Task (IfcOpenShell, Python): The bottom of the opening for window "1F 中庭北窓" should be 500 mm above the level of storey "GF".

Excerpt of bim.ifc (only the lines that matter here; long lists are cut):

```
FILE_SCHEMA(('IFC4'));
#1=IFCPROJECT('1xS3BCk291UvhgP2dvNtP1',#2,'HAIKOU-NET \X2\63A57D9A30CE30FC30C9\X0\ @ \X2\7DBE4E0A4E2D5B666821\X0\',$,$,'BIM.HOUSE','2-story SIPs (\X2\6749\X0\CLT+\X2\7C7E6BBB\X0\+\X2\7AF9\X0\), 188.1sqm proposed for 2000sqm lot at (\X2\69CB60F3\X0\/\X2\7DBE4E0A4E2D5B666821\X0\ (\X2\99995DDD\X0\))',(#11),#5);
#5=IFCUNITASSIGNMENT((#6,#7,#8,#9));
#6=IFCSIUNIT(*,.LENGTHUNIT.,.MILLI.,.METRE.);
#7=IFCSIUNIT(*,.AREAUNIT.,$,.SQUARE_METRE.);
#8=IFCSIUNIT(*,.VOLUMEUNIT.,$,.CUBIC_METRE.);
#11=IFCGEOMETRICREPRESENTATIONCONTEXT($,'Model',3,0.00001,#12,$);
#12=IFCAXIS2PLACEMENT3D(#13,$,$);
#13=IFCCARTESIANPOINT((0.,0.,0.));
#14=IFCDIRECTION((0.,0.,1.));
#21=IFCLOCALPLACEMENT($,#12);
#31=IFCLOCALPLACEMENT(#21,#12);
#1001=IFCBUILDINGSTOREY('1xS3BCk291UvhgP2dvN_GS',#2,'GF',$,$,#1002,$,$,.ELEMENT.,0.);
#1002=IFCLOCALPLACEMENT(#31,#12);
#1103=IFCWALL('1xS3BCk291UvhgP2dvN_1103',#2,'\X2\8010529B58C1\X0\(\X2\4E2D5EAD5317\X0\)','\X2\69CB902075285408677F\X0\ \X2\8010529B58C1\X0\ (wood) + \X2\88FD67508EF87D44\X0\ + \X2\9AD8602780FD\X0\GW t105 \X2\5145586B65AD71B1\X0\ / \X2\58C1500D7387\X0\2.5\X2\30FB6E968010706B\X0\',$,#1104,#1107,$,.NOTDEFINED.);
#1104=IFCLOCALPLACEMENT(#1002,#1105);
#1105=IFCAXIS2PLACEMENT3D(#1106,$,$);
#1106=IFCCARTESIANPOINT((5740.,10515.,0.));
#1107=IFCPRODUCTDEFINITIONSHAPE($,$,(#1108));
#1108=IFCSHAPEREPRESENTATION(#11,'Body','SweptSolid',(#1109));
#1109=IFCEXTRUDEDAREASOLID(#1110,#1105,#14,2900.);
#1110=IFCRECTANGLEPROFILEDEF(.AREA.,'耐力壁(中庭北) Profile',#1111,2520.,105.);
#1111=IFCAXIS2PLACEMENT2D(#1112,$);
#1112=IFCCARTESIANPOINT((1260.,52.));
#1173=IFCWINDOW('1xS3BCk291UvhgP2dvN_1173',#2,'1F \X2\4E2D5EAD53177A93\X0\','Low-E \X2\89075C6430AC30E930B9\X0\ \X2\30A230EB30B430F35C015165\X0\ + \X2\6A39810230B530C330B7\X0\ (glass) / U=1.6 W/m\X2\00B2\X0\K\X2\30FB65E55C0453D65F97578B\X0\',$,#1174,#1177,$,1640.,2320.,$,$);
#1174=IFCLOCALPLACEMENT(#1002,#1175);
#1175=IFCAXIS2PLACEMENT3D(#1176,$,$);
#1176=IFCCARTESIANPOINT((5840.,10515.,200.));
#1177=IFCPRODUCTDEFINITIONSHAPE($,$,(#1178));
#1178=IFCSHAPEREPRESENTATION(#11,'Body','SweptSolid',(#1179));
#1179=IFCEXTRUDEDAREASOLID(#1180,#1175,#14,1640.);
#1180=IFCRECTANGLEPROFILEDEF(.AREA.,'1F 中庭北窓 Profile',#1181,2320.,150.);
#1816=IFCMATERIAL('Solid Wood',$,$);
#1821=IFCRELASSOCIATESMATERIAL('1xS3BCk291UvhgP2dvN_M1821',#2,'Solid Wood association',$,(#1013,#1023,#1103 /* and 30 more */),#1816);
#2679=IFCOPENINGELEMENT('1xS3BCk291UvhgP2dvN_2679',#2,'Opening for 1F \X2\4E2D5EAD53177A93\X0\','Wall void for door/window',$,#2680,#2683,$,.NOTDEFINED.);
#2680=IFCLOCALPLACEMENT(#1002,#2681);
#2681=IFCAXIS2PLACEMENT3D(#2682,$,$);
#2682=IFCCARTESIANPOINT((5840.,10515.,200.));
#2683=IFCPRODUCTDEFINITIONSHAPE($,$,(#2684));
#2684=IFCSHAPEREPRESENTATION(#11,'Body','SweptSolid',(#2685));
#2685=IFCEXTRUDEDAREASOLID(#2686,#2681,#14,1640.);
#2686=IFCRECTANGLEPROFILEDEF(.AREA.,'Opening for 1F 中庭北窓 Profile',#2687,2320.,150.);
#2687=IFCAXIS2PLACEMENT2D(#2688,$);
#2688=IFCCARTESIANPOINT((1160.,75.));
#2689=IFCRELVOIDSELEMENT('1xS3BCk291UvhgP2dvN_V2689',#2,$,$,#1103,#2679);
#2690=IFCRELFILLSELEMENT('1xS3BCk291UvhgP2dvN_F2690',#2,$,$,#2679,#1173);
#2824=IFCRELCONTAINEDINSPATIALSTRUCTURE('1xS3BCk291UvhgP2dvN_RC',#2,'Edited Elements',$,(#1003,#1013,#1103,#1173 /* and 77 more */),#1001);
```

```python
import numpy as np
import ifcopenshell
import ifcopenshell.api.geometry
import ifcopenshell.geom
import ifcopenshell.util.element
import ifcopenshell.util.placement
import ifcopenshell.util.shape
import ifcopenshell.util.unit

model = ifcopenshell.open("bim.ifc")
unit_scale = ifcopenshell.util.unit.calculate_unit_scale(model)

window = model.by_guid("1xS3BCk291UvhgP2dvN_1173")
opening = window.FillsVoids[0].RelatingOpeningElement
storey = ifcopenshell.util.element.get_container(window, ifc_class="IfcBuildingStorey")
level = ifcopenshell.util.placement.get_local_placement(storey.ObjectPlacement)[2, 3]

# The opening's origin need not be at the sill, so measure its lowest point.
shape = ifcopenshell.geom.create_shape(ifcopenshell.geom.settings(), opening)
bottom = ifcopenshell.util.shape.get_shape_bottom_elevation(shape, shape.geometry) / unit_scale
dz = level + 500.0 - bottom

shift = np.array([0.0, 0.0, dz])
# The window is not placed relative to its opening, so move both.
for product in (opening, window):
    matrix = ifcopenshell.util.placement.get_local_placement(product.ObjectPlacement)
    matrix[:3, 3] += shift
    ifcopenshell.api.geometry.edit_object_placement(model, product=product, matrix=matrix, is_si=False)

print(f"moved by {dz * unit_scale:+.3f} m")

model.write("bim_rev.ifc")
```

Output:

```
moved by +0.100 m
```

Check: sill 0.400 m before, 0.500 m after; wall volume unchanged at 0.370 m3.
